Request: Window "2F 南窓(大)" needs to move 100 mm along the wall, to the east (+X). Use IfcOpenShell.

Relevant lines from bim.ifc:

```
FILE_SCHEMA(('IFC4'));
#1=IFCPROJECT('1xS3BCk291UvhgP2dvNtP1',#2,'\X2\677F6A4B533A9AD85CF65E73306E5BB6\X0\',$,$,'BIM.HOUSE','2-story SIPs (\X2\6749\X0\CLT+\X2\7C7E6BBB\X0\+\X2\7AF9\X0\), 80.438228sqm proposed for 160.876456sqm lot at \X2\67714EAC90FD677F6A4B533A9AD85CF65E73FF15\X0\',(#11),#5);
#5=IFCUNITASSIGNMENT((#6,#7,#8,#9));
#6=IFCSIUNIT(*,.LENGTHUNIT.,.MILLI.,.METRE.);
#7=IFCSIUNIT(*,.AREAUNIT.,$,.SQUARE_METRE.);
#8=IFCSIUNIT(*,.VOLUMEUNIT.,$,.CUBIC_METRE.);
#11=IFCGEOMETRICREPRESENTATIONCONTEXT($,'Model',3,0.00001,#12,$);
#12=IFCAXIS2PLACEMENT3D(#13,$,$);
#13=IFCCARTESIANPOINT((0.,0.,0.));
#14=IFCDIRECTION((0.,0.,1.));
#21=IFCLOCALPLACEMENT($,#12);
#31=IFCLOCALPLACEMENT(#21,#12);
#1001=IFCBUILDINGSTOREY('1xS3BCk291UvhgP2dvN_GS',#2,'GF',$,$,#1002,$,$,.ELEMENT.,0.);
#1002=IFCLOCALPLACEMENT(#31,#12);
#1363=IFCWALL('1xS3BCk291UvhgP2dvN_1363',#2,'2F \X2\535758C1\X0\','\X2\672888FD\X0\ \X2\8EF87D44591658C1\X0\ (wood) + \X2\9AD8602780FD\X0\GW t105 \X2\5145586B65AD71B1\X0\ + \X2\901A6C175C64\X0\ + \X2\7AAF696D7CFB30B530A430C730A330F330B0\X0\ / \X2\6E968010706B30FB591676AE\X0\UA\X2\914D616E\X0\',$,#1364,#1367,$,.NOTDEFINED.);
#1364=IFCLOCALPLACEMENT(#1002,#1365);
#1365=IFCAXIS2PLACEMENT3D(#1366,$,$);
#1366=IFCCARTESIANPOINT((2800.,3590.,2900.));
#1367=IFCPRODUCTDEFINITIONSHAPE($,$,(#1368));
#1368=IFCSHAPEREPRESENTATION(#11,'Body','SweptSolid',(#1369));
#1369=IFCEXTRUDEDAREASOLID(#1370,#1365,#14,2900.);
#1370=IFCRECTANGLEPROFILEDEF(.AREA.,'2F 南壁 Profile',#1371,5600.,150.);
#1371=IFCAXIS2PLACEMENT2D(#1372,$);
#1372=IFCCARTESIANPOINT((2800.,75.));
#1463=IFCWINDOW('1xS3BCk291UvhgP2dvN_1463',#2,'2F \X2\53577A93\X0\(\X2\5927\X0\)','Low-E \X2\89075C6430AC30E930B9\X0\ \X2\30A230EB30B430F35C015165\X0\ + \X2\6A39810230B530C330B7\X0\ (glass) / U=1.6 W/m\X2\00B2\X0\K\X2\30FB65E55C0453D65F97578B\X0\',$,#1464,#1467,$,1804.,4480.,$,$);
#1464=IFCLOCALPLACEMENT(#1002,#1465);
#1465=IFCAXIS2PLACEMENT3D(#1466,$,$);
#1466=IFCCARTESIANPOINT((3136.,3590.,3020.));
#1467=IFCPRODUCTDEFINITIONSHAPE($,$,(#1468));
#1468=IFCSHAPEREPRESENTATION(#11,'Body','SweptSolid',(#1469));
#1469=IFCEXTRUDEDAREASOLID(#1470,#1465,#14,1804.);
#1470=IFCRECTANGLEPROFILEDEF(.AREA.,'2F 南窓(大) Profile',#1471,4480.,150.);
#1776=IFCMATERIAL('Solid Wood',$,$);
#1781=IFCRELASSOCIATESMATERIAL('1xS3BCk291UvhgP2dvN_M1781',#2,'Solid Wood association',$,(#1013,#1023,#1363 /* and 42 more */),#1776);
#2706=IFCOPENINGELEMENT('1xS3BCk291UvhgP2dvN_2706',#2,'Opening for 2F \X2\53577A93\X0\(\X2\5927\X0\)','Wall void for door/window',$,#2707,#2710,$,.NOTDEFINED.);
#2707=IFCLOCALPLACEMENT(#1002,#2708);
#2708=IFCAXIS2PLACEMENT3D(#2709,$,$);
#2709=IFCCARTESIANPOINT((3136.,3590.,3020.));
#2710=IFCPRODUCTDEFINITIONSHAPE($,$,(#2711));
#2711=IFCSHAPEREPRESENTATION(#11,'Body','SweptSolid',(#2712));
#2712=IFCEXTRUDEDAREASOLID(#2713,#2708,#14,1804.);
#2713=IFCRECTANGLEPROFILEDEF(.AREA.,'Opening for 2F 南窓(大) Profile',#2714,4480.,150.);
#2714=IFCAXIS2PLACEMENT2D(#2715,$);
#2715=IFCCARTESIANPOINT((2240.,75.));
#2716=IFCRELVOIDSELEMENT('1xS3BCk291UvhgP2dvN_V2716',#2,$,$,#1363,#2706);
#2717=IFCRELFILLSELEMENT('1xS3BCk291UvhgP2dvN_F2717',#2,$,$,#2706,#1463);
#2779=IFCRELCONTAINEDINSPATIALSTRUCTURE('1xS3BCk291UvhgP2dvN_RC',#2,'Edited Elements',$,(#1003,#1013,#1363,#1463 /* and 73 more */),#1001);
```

```python
import ifcopenshell
import ifcopenshell.api.geometry
import ifcopenshell.util.placement

model = ifcopenshell.open("bim.ifc")

window = model.by_guid("1xS3BCk291UvhgP2dvN_1463")
opening = window.FillsVoids[0].RelatingOpeningElement
wall = opening.VoidsElements[0].RelatingBuildingElement

wall_matrix = ifcopenshell.util.placement.get_local_placement(wall.ObjectPlacement)
shift = wall_matrix[:3, 0] * 100.0
before = ifcopenshell.util.placement.get_local_placement(window.ObjectPlacement)[:3, 3].copy()

# The window is not placed relative to its opening, so move both.
for product in (opening, window):
    matrix = ifcopenshell.util.placement.get_local_placement(product.ObjectPlacement)
    matrix[:3, 3] += shift
    ifcopenshell.api.geometry.edit_object_placement(model, product=product, matrix=matrix, is_si=False)

after = ifcopenshell.util.placement.get_local_placement(window.ObjectPlacement)[:3, 3]
print("window moved by", (after - before).round(3) + 0.0)

model.write("bim_rev.ifc")
```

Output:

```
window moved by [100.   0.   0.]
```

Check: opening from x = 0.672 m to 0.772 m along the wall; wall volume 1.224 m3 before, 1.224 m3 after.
